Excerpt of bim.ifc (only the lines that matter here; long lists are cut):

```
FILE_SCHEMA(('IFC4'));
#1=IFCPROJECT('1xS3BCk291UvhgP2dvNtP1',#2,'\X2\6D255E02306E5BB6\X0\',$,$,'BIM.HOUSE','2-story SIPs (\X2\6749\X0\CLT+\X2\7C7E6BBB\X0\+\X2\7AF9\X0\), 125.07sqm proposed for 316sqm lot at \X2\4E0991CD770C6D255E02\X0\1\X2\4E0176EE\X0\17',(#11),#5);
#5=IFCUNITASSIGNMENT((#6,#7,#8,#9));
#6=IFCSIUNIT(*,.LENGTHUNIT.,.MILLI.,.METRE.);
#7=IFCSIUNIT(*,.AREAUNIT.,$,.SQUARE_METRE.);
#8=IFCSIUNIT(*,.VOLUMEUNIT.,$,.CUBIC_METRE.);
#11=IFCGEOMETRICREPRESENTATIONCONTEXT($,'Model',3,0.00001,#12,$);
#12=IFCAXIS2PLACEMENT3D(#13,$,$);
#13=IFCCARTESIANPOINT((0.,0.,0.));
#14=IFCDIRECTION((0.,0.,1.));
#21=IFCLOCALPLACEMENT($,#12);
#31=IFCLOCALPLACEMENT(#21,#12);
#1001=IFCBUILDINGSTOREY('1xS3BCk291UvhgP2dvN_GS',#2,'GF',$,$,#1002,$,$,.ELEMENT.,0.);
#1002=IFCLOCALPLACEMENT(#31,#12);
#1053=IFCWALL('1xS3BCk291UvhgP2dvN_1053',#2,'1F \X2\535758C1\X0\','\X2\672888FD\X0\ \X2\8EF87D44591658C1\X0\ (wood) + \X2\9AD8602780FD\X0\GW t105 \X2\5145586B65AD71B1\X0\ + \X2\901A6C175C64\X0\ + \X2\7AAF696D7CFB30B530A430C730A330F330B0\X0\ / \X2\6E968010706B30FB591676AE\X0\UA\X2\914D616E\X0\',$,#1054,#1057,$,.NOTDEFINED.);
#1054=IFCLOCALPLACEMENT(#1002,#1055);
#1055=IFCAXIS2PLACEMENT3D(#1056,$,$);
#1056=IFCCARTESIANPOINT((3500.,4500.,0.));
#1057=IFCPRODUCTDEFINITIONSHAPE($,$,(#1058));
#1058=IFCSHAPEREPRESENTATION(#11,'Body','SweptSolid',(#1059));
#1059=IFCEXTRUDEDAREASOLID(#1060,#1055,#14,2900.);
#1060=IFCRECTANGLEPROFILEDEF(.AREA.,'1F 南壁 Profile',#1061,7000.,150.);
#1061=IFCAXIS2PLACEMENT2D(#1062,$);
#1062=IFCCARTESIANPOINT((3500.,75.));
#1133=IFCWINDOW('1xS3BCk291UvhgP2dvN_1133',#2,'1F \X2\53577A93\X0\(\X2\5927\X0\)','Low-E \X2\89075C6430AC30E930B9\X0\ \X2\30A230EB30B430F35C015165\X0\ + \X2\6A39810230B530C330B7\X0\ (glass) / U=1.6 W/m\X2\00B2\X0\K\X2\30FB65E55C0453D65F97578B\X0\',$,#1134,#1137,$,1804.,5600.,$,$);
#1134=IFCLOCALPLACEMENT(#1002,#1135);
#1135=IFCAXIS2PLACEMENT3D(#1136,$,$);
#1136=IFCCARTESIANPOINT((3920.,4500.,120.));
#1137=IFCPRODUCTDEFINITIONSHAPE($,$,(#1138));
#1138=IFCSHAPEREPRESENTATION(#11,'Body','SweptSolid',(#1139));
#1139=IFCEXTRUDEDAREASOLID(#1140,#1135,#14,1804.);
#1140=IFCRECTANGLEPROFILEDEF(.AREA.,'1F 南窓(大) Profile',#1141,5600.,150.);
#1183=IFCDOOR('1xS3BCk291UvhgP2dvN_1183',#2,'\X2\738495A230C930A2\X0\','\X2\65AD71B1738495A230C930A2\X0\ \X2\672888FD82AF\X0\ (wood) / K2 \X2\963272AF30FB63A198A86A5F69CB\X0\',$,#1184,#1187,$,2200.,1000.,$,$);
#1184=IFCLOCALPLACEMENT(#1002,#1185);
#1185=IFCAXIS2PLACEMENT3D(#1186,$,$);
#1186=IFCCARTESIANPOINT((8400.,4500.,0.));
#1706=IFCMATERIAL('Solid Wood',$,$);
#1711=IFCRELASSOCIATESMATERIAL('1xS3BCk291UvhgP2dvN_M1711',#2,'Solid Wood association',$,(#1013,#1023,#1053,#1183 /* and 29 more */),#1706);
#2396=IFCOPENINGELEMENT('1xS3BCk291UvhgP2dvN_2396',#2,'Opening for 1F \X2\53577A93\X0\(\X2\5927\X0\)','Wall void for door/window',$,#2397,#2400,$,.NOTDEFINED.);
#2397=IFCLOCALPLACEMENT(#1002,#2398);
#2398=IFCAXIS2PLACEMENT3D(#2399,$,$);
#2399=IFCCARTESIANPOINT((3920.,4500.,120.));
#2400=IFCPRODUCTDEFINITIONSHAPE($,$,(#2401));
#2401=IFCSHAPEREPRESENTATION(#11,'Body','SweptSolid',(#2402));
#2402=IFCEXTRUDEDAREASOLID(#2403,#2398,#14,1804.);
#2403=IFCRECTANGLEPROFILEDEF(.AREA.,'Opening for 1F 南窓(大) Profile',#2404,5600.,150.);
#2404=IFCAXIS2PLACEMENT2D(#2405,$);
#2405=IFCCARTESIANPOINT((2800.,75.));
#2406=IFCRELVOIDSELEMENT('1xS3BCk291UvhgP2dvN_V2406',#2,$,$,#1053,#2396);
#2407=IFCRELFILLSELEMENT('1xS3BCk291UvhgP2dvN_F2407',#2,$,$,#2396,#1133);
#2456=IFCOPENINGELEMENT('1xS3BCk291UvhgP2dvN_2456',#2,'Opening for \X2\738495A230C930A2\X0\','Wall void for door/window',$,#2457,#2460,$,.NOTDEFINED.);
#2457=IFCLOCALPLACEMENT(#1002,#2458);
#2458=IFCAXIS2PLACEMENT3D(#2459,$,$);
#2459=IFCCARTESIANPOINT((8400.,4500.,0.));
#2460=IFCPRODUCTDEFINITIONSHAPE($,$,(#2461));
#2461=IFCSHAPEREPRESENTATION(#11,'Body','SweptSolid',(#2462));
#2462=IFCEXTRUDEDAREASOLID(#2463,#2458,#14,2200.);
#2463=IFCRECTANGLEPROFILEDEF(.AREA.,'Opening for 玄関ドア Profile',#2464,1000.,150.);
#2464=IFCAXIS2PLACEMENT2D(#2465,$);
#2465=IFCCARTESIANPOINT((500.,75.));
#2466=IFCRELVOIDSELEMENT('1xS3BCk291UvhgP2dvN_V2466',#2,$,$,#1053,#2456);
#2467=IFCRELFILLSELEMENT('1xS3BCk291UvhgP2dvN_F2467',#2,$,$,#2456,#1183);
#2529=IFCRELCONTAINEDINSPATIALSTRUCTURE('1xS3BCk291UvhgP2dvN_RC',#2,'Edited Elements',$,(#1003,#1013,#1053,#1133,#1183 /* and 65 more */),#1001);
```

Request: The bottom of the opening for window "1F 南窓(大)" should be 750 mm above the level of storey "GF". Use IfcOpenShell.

```python
import numpy as np
import ifcopenshell
import ifcopenshell.api.geometry
import ifcopenshell.geom
import ifcopenshell.util.element
import ifcopenshell.util.placement
import ifcopenshell.util.shape
import ifcopenshell.util.unit

model = ifcopenshell.open("bim.ifc")
unit_scale = ifcopenshell.util.unit.calculate_unit_scale(model)

window = model.by_id(1133)
opening = window.FillsVoids[0].RelatingOpeningElement
storey = ifcopenshell.util.element.get_container(window, ifc_class="IfcBuildingStorey")
level = ifcopenshell.util.placement.get_local_placement(storey.ObjectPlacement)[2, 3]

# The opening's origin need not be at the sill, so measure its lowest point.
shape = ifcopenshell.geom.create_shape(ifcopenshell.geom.settings(), opening)
bottom = ifcopenshell.util.shape.get_shape_bottom_elevation(shape, shape.geometry) / unit_scale
dz = level + 0.75 / unit_scale - bottom

shift = np.array([0.0, 0.0, dz])
# The window is not placed relative to its opening, so move both.
for product in (opening, window):
    matrix = ifcopenshell.util.placement.get_local_placement(product.ObjectPlacement)
    matrix[:3, 3] += shift
    ifcopenshell.api.geometry.edit_object_placement(model, product=product, matrix=matrix, is_si=False)

print(f"moved by {dz * unit_scale:+.3f} m")

model.write("bim_edited.ifc")
```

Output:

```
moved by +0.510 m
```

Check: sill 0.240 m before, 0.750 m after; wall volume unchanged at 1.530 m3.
